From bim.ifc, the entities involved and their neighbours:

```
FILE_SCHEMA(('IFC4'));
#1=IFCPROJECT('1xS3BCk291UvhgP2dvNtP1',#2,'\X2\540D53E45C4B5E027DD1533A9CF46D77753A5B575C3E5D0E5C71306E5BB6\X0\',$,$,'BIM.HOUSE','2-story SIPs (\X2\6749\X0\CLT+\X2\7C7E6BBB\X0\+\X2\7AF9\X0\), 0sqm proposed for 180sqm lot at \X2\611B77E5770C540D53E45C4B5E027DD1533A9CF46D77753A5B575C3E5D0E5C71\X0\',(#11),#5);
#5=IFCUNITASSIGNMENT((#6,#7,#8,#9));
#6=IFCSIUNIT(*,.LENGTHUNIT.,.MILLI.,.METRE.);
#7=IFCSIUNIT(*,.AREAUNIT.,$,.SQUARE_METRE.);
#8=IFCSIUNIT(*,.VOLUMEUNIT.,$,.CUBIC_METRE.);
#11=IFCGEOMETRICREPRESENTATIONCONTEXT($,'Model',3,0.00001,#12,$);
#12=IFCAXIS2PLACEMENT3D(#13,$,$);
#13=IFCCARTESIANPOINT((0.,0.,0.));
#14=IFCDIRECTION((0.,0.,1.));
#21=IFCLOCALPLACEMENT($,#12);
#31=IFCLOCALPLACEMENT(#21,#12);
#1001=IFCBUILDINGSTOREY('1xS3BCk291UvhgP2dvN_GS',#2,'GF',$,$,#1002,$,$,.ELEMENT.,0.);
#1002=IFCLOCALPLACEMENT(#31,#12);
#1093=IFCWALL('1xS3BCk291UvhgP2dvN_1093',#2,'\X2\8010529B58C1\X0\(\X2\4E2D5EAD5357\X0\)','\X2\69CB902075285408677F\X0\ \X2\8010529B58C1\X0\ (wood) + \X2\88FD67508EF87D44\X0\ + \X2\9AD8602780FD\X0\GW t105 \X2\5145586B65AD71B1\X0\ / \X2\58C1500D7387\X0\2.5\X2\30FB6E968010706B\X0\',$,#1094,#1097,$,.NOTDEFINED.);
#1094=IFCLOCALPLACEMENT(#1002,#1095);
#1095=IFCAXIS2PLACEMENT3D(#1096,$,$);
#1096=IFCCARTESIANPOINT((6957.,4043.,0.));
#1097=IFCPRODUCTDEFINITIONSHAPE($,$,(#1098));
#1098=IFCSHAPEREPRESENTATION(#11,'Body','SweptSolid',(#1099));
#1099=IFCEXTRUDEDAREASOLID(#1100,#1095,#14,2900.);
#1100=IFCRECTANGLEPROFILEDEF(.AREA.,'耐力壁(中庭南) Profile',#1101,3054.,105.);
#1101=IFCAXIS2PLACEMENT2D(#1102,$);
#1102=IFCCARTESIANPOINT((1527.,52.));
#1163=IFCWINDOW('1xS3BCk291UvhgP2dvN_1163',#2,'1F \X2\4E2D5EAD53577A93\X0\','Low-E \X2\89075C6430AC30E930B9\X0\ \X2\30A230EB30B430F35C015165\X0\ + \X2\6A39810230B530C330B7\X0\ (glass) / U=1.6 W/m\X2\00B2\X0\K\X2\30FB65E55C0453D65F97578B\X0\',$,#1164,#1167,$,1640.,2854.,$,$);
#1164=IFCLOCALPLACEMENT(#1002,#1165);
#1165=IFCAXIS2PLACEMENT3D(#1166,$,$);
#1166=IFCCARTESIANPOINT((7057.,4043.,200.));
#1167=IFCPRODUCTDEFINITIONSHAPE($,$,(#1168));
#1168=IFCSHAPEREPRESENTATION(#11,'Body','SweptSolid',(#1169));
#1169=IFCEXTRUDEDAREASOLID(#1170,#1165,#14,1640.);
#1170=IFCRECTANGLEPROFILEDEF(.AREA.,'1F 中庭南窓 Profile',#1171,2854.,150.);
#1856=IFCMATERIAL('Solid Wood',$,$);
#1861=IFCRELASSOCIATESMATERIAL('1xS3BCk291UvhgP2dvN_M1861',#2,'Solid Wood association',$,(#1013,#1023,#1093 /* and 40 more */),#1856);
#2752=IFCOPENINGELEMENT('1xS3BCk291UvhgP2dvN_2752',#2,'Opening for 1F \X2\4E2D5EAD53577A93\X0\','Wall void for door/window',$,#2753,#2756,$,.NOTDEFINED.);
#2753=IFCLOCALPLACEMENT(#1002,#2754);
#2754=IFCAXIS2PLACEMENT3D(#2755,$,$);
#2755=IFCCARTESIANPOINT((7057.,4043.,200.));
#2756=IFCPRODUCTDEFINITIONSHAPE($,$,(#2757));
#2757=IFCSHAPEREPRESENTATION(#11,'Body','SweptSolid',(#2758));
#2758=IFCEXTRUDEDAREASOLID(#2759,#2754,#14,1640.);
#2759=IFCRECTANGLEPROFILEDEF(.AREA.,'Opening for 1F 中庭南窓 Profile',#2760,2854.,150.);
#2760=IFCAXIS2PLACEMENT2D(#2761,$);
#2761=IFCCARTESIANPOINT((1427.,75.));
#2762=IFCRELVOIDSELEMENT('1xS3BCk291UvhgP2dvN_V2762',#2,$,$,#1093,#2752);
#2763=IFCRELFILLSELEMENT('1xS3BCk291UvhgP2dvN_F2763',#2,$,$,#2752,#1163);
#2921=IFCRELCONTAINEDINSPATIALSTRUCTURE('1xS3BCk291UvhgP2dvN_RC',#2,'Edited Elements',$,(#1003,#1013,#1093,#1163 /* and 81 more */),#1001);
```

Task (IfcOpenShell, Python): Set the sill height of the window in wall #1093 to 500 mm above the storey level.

```python
import numpy as np
import ifcopenshell
import ifcopenshell.api.geometry
import ifcopenshell.geom
import ifcopenshell.util.element
import ifcopenshell.util.placement
import ifcopenshell.util.shape
import ifcopenshell.util.unit

model = ifcopenshell.open("bim.ifc")
unit_scale = ifcopenshell.util.unit.calculate_unit_scale(model)

window = model.by_id(1163)
opening = window.FillsVoids[0].RelatingOpeningElement
storey = ifcopenshell.util.element.get_container(window, ifc_class="IfcBuildingStorey")
level = ifcopenshell.util.placement.get_local_placement(storey.ObjectPlacement)[2, 3]

# The opening's origin need not be at the sill, so measure its lowest point.
shape = ifcopenshell.geom.create_shape(ifcopenshell.geom.settings(), opening)
bottom = ifcopenshell.util.shape.get_shape_bottom_elevation(shape, shape.geometry) / unit_scale
dz = level + 500.0 - bottom

shift = np.array([0.0, 0.0, dz])
# The window is not placed relative to its opening, so move both.
for product in (opening, window):
    matrix = ifcopenshell.util.placement.get_local_placement(product.ObjectPlacement)
    matrix[:3, 3] += shift
    ifcopenshell.api.geometry.edit_object_placement(model, product=product, matrix=matrix, is_si=False)

print(f"moved by {dz * unit_scale:+.3f} m")

model.write("bim_updated.ifc")
```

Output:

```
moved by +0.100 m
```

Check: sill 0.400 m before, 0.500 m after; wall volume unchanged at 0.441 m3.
